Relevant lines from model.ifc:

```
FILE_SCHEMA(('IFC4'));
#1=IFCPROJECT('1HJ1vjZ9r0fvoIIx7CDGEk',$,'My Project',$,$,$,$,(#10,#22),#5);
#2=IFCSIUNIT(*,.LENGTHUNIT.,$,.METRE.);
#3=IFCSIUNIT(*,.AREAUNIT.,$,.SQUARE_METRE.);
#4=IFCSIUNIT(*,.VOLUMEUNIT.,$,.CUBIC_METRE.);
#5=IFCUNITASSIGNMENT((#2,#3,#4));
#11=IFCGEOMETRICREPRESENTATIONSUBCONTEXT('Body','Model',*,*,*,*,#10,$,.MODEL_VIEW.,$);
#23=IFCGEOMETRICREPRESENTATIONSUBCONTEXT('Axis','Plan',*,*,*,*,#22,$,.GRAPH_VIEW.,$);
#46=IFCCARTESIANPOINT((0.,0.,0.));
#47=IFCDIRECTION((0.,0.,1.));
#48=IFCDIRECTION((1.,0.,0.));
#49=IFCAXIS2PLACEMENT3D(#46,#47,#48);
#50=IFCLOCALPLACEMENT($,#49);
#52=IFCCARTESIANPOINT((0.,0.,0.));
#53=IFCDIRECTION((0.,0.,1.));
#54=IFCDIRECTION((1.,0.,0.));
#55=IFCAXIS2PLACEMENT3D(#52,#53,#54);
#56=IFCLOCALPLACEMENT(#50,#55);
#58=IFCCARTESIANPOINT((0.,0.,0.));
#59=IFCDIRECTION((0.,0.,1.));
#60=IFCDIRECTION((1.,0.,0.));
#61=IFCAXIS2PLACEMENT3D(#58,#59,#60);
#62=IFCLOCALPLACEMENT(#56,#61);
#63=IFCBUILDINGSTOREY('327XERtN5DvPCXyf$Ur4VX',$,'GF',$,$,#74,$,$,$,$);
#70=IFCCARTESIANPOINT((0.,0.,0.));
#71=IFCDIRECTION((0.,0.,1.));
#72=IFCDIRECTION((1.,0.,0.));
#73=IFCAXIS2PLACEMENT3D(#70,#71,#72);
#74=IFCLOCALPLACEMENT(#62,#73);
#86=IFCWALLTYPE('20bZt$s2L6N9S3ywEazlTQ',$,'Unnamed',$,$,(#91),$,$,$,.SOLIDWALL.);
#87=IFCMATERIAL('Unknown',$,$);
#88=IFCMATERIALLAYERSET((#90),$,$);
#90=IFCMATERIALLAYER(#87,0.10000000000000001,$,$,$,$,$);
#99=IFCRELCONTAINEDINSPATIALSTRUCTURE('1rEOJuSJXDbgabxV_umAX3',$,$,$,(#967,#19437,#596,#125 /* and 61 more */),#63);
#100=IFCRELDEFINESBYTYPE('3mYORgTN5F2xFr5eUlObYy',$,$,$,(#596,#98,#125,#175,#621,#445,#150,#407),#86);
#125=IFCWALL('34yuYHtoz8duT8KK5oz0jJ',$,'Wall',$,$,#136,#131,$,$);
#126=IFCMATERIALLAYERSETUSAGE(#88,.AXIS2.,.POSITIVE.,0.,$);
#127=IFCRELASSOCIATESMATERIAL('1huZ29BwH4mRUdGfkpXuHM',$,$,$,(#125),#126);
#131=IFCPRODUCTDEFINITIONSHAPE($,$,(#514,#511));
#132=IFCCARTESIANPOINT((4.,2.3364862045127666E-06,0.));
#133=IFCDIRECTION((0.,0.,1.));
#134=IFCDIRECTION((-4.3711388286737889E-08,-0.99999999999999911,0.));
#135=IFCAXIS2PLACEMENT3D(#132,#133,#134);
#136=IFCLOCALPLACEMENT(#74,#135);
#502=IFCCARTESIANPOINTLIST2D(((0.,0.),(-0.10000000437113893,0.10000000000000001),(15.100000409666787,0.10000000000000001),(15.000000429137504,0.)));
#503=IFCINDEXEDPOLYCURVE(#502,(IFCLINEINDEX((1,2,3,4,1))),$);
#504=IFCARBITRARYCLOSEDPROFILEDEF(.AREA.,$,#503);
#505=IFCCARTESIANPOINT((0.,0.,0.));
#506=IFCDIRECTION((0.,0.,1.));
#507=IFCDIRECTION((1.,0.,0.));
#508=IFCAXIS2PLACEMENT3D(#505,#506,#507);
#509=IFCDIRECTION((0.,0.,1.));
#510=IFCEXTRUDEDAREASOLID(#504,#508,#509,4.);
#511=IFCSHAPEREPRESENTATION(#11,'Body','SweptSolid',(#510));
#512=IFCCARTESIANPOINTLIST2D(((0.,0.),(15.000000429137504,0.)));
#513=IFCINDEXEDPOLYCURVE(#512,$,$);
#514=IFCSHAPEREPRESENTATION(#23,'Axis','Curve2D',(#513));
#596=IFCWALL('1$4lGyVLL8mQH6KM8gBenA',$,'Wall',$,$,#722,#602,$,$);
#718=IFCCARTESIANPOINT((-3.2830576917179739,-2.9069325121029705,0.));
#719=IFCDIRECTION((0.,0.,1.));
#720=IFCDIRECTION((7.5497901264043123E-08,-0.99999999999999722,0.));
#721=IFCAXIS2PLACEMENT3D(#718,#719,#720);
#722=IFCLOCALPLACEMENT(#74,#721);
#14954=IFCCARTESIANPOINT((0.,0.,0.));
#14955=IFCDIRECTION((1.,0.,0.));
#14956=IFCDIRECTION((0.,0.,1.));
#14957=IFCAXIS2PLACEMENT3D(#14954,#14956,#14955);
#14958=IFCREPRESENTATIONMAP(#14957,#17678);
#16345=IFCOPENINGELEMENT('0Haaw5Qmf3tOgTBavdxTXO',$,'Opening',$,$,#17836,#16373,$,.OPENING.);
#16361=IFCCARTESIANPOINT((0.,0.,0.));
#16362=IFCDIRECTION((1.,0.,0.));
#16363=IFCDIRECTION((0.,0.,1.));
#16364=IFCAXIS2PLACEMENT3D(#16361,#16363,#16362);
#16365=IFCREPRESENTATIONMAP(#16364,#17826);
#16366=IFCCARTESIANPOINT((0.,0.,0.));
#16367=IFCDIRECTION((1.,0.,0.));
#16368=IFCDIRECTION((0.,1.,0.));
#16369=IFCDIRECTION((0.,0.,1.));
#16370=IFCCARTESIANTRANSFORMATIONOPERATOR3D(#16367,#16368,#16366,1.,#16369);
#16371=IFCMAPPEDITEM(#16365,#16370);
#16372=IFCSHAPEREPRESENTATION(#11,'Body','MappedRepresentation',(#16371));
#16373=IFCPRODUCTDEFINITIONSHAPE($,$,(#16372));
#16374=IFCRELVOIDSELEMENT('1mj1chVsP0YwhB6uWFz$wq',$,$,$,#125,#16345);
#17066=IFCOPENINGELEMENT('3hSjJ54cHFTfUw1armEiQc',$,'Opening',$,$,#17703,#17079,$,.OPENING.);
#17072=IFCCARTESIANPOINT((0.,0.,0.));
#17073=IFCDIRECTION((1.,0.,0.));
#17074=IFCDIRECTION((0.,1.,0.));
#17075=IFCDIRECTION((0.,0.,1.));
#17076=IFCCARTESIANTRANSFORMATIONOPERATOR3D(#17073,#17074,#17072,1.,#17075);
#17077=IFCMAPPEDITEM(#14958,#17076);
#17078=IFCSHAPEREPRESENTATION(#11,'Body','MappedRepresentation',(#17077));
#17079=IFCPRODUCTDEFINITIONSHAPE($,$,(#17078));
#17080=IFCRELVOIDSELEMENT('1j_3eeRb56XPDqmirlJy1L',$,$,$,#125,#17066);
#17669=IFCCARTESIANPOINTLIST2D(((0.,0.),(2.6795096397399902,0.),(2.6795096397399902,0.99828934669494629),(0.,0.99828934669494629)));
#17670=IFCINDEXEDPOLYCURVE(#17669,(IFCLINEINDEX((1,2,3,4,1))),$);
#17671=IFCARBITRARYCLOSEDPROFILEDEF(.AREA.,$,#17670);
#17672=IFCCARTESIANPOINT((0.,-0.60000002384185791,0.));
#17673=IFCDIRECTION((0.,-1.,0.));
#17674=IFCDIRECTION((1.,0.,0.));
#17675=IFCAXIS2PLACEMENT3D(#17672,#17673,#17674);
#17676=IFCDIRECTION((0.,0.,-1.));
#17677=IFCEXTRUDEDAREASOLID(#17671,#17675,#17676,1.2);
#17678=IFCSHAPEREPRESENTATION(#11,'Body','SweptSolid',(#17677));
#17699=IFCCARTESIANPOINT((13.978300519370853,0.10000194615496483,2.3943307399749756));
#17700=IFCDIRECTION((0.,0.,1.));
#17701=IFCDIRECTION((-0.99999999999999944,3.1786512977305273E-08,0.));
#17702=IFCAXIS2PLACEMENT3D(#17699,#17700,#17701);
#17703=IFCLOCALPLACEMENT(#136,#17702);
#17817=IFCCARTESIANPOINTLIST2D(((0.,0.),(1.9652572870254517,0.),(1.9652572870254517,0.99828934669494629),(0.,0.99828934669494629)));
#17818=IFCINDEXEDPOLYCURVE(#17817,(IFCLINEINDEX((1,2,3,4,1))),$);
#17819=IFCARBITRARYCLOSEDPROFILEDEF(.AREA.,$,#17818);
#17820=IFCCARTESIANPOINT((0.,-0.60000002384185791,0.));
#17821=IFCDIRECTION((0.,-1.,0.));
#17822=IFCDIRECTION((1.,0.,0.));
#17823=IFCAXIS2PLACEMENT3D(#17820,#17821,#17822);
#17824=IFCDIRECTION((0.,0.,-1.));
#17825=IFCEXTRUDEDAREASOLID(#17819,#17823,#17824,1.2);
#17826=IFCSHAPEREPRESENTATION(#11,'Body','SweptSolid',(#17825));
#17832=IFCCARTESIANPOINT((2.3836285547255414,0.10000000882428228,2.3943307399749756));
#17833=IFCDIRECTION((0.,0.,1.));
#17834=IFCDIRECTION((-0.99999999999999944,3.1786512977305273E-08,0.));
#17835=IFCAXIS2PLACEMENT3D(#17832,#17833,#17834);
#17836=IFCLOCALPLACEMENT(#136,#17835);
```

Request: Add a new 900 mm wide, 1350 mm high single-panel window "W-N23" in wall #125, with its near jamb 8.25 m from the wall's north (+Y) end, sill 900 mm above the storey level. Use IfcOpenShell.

```python
import numpy as np
import ifcopenshell
import ifcopenshell.api.feature
import ifcopenshell.api.geometry
import ifcopenshell.api.root
import ifcopenshell.api.spatial
import ifcopenshell.geom
import ifcopenshell.util.element
import ifcopenshell.util.placement
import ifcopenshell.util.representation
import ifcopenshell.util.shape
import ifcopenshell.util.unit

model = ifcopenshell.open("model.ifc")
unit_scale = ifcopenshell.util.unit.calculate_unit_scale(model)
settings = ifcopenshell.geom.settings()


def volume(element):
    """Net volume in cubic metres, openings subtracted."""
    shape = ifcopenshell.geom.create_shape(settings, element)
    return ifcopenshell.util.shape.get_volume(shape.geometry)


wall = model.by_guid("34yuYHtoz8duT8KK5oz0jJ")
storey = ifcopenshell.util.element.get_container(wall, ifc_class="IfcBuildingStorey")
context = ifcopenshell.util.representation.get_context(model, "Model", "Body", "MODEL_VIEW")
before = volume(wall)

width, height, from_end, sill = 0.9, 1.35, 8.25, 0.9  # metres

# The wall runs along its own X axis, and the end named is its -X end.
wall_shape = ifcopenshell.geom.create_shape(settings, wall)
x, y, z = ifcopenshell.util.shape.get_vertices(wall_shape.geometry).T
start = x.min() + from_end
face, thickness = float(y.min()), float(y.max() - y.min())
wall_matrix = ifcopenshell.util.placement.get_local_placement(wall.ObjectPlacement)
level = ifcopenshell.util.placement.get_local_placement(storey.ObjectPlacement)[2, 3]


def in_wall(x, y):
    """Placement at x, y metres in the wall's axes, at sill height."""
    matrix = wall_matrix.copy()
    matrix[:, 3] = wall_matrix @ np.array([x / unit_scale, y / unit_scale, 0.0, 1.0])
    matrix[2, 3] = level + sill / unit_scale
    return matrix


# Opening: a box that overshoots both wall faces by 50 mm.
opening = ifcopenshell.api.root.create_entity(model, ifc_class="IfcOpeningElement", predefined_type="OPENING")
box = ifcopenshell.api.geometry.add_wall_representation(
    model, context=context, length=width, height=height, thickness=thickness + 0.1
)
ifcopenshell.api.geometry.assign_representation(model, product=opening, representation=box)
ifcopenshell.api.geometry.edit_object_placement(model, product=opening, matrix=in_wall(start, face - 0.05), is_si=False)
ifcopenshell.api.feature.add_feature(model, feature=opening, element=wall)

window = ifcopenshell.api.root.create_entity(model, ifc_class="IfcWindow", name="W-N23", predefined_type="WINDOW")
window.OverallWidth, window.OverallHeight = width / unit_scale, height / unit_scale
window.PartitioningType = "SINGLE_PANEL"
body = ifcopenshell.api.geometry.add_window_representation(
    model,
    context=context,
    overall_width=window.OverallWidth,
    overall_height=window.OverallHeight,
    partition_type="SINGLE_PANEL",
)
ifcopenshell.api.geometry.assign_representation(model, product=window, representation=body)
ifcopenshell.api.spatial.assign_container(model, products=[window], relating_structure=storey)
ifcopenshell.api.feature.add_filling(model, opening=opening, element=window)

# Centre the window in the wall's thickness.
ifcopenshell.api.geometry.edit_object_placement(model, product=window, matrix=in_wall(start, face), is_si=False)
window_shape = ifcopenshell.geom.create_shape(settings, window)
depth = ifcopenshell.util.shape.get_vertices(window_shape.geometry)[:, 1]
offset = face + thickness / 2 - (depth.min() + depth.max()) / 2
ifcopenshell.api.geometry.edit_object_placement(model, product=window, matrix=in_wall(start, offset), is_si=False)

after = volume(wall)

print(f"wall volume {before:.3f} -> {after:.3f} m3")

model.write("model-out.ifc")
```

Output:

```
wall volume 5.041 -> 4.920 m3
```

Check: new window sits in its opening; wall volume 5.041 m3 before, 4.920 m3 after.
